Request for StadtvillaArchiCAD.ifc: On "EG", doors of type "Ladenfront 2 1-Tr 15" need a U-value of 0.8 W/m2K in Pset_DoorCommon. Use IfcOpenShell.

First a look at what the model holds.

```python
import ifcopenshell
import ifcopenshell.util.element

model = ifcopenshell.open("StadtvillaArchiCAD.ifc")
print(model.schema)
storey = next(s for s in model.by_type("IfcBuildingStorey") if s.Name == "EG")
doors = [e for e in ifcopenshell.util.element.get_decomposition(storey) if e.is_a("IfcDoor")]
seen = {}
for e in doors:
    element_type = ifcopenshell.util.element.get_type(e)
    key = (element_type.Name if element_type != e and element_type else None, ifcopenshell.util.element.get_pset(e, "Pset_DoorCommon", "ThermalTransmittance"))
    seen[key] = seen.get(key, 0) + 1
for (name, value), count in sorted(seen.items(), key=str):
    print(count, "x", name, "|", value)
```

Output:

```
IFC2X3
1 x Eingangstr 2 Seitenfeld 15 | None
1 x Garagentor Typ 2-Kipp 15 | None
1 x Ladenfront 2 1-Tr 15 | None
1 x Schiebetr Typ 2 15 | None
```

```python
import ifcopenshell
import ifcopenshell.api.pset
import ifcopenshell.util.element

model = ifcopenshell.open("StadtvillaArchiCAD.ifc")

storey = next(s for s in model.by_type("IfcBuildingStorey") if s.Name == "EG")
doors = [e for e in ifcopenshell.util.element.get_decomposition(storey) if e.is_a("IfcDoor")]

count = 0
for e in doors:
    element_type = ifcopenshell.util.element.get_type(e)
    if element_type in (None, e) or element_type.Name != 'Ladenfront 2 1-T\x9fr 15':
        continue
    # add_pset returns the element's existing set when there is one.
    pset = ifcopenshell.api.pset.add_pset(model, product=e, name="Pset_DoorCommon")
    ifcopenshell.api.pset.edit_pset(model, pset=pset, properties={"ThermalTransmittance": 0.8})
    count += 1

print(count, "doors updated")

model.write("StadtvillaArchiCAD-out.ifc")
```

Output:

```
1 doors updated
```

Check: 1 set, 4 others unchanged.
